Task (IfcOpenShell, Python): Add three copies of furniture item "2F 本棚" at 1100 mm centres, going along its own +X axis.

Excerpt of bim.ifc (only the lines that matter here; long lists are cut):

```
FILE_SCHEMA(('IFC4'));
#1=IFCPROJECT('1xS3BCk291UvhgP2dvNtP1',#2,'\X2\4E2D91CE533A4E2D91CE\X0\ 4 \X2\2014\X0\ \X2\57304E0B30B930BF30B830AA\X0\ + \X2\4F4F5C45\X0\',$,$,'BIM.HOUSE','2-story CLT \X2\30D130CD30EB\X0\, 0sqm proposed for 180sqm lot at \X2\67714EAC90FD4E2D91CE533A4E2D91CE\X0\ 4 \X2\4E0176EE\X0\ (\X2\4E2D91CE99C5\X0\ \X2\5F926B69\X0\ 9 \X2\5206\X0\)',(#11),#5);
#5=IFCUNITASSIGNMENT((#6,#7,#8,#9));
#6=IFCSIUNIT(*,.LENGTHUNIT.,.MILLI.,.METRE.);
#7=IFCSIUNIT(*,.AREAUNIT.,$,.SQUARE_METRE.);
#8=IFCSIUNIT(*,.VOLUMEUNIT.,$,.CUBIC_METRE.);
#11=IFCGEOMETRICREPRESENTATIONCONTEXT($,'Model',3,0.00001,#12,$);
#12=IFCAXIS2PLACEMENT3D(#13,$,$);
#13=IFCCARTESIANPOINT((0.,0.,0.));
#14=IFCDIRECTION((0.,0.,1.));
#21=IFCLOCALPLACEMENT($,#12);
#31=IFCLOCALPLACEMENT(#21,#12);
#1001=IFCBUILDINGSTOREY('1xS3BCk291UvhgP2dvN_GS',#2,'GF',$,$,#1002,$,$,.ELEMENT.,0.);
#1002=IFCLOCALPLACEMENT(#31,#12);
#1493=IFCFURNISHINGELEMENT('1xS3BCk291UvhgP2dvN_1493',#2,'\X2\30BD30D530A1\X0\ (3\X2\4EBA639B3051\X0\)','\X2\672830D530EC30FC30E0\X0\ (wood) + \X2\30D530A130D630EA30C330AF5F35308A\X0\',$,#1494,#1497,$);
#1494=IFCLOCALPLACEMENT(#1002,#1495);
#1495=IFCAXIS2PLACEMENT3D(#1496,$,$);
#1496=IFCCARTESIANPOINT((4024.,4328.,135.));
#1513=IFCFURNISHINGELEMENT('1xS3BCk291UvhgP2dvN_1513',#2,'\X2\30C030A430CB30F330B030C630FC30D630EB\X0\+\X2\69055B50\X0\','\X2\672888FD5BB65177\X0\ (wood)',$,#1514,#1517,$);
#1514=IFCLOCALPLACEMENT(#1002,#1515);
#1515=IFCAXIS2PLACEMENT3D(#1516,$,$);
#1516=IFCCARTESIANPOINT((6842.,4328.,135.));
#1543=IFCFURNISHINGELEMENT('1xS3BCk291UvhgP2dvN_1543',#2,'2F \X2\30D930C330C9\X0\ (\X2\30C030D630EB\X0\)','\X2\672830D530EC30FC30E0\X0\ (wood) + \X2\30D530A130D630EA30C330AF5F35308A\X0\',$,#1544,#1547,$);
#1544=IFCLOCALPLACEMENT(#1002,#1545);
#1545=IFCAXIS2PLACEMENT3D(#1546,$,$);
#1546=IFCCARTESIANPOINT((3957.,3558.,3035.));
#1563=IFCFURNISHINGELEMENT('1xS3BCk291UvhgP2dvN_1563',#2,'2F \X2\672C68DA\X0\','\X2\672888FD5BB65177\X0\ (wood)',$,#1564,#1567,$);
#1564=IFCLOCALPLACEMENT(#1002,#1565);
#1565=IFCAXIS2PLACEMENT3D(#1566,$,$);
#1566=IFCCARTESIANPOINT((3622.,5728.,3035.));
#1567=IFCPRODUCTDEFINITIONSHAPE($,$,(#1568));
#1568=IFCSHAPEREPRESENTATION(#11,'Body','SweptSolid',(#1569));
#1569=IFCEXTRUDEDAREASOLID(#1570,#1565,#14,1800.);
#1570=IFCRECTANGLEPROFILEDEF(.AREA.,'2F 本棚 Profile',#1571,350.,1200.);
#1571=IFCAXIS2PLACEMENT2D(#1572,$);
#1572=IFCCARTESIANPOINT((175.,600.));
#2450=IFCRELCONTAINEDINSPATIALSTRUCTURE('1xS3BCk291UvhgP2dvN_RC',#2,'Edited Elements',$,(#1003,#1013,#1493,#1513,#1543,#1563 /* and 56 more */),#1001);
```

```python
import ifcopenshell
import ifcopenshell.api.geometry
import ifcopenshell.api.root
import ifcopenshell.util.element
import ifcopenshell.util.placement

model = ifcopenshell.open("bim.ifc")


def reuse_history(source, copy):
    """copy_class also copies each property set's owner history, people and application; keep the originals."""
    for rel in copy.IsDefinedBy:
        if rel.is_a("IfcRelDefinesByProperties") and (history := rel.RelatingPropertyDefinition.OwnerHistory):
            rel.RelatingPropertyDefinition.OwnerHistory = source.OwnerHistory
            ifcopenshell.util.element.remove_deep2(model, history)


source = model.by_guid("1xS3BCk291UvhgP2dvN_1563")
base = ifcopenshell.util.placement.get_local_placement(source.ObjectPlacement)
step = base[:3, 0] * 1100.0

for i in range(1, 4):
    copy = ifcopenshell.api.root.copy_class(model, product=source)
    copy.Representation = ifcopenshell.util.element.copy_deep(
        model, source.Representation, exclude=["IfcGeometricRepresentationContext", "IfcRepresentationMap"]
    )
    reuse_history(source, copy)
    matrix = base.copy()
    matrix[:3, 3] += i * step
    print("added at", matrix[:3, 3].round(3) + 0.0)
    ifcopenshell.api.geometry.edit_object_placement(model, product=copy, matrix=matrix, is_si=False)

model.write("bim_rev.ifc")
```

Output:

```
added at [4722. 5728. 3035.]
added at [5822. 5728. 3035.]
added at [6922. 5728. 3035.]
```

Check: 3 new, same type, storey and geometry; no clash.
